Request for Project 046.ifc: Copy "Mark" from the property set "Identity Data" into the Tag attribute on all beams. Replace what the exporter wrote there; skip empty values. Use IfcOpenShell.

First a look at what the model holds.

```python
import ifcopenshell
import ifcopenshell.util.element

model = ifcopenshell.open("Project 046.ifc")
print(model.schema)
beams = model.by_type("IfcBeam")
print(len(beams), "beams")
for e in beams[:8]:
    source = ifcopenshell.util.element.get_pset(e, "Identity Data", "Mark")
    target = e.Tag
    print(e.id(), repr(source), repr(target), sep=" | ")
```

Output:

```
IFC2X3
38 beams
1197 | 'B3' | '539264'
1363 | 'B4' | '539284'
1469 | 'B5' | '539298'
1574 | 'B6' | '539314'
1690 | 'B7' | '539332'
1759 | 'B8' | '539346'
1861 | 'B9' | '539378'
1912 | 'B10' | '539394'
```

```python
import ifcopenshell
import ifcopenshell.util.element

model = ifcopenshell.open("Project 046.ifc")

count = 0
for e in model.by_type("IfcBeam"):
    value = ifcopenshell.util.element.get_pset(e, "Identity Data", "Mark")
    current = e.Tag
    if not value or not value.strip() or current == value:
        continue
    e.Tag = value
    count += 1

print(count, "beams updated")

model.write("Project 046_rev.ifc")
```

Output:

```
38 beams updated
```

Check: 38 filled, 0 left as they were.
